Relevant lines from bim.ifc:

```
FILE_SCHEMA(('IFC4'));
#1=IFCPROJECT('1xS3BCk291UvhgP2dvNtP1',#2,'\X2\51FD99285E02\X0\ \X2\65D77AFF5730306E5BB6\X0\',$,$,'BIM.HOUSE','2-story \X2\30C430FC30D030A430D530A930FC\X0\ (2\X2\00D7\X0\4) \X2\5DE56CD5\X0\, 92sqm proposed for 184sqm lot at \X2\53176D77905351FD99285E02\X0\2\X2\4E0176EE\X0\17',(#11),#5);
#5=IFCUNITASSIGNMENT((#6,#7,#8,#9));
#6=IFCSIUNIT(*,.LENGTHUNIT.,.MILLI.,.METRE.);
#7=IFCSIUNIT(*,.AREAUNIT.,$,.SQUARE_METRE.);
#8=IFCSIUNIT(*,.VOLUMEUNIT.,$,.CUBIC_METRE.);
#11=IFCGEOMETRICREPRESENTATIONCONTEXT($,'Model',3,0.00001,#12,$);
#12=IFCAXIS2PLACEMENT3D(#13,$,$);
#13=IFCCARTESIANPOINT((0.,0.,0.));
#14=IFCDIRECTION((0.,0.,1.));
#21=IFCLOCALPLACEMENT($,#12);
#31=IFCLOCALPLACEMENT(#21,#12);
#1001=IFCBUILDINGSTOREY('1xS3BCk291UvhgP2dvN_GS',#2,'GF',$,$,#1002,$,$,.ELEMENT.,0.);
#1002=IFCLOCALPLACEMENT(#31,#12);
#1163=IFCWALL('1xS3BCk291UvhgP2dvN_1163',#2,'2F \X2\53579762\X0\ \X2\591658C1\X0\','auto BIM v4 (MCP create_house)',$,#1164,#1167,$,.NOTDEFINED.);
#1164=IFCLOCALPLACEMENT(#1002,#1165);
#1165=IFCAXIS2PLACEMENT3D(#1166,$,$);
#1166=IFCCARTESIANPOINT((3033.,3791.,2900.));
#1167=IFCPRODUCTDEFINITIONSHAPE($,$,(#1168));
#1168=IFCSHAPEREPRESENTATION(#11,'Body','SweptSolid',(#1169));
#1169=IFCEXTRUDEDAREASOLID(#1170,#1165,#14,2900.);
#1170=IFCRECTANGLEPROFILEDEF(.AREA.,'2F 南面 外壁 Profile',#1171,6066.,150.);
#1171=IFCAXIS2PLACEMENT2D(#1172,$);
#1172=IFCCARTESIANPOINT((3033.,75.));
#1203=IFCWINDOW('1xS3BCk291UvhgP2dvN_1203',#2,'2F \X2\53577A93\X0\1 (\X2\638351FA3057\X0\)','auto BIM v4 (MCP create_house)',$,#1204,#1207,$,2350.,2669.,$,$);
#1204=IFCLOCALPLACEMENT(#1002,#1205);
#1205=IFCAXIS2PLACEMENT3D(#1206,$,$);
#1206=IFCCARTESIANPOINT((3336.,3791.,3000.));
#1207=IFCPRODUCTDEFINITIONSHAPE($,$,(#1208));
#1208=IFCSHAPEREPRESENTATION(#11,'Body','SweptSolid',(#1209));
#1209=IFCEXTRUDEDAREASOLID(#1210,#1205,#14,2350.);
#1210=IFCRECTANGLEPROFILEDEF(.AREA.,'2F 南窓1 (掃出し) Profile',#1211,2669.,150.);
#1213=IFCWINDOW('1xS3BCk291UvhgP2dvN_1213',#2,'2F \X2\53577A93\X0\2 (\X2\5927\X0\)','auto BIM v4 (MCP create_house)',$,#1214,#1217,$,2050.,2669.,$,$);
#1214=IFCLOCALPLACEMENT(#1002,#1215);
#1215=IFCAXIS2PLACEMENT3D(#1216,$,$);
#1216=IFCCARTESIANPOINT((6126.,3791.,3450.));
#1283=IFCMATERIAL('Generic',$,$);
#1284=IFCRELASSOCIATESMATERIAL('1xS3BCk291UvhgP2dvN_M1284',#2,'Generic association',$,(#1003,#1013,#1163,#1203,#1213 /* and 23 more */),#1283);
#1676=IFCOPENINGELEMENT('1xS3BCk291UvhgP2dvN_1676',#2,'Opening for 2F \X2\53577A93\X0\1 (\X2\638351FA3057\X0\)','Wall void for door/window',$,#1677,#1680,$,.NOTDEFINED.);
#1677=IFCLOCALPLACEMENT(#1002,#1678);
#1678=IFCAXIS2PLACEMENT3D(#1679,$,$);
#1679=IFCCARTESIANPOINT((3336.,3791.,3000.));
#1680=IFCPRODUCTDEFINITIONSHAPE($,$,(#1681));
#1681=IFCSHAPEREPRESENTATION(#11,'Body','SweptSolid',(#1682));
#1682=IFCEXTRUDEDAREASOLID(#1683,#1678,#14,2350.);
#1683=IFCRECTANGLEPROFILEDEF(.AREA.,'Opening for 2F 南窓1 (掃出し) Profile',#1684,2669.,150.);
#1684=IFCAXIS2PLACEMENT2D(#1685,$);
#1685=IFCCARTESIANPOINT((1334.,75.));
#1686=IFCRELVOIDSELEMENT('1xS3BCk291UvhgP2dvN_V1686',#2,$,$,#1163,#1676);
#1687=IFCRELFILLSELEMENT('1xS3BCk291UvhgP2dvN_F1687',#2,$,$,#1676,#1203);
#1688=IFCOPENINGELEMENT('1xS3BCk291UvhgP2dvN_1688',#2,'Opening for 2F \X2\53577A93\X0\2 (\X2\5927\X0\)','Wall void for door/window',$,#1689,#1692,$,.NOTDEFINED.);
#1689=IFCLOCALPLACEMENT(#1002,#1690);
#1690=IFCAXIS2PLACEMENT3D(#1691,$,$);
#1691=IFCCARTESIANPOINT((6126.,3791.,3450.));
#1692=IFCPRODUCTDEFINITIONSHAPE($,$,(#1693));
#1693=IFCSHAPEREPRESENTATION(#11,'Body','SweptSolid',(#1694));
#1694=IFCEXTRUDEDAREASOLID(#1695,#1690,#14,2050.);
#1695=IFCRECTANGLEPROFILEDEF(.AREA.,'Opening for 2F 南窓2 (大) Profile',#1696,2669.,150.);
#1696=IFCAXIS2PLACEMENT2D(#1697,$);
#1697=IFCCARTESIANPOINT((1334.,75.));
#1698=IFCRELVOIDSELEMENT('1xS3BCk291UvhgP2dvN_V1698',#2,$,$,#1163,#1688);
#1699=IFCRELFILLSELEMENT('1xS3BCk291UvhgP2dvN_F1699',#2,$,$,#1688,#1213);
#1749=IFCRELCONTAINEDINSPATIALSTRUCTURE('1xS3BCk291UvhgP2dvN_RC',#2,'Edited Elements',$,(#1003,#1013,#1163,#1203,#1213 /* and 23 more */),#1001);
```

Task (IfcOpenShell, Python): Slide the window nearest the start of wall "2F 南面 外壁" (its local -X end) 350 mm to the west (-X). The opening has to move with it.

```python
import ifcopenshell
import ifcopenshell.api.geometry
import ifcopenshell.util.placement
import ifcopenshell.util.unit

model = ifcopenshell.open("bim.ifc")
unit_scale = ifcopenshell.util.unit.calculate_unit_scale(model)

window = model.by_guid("1xS3BCk291UvhgP2dvN_1203")
opening = window.FillsVoids[0].RelatingOpeningElement
wall = opening.VoidsElements[0].RelatingBuildingElement

wall_matrix = ifcopenshell.util.placement.get_local_placement(wall.ObjectPlacement)
shift = wall_matrix[:3, 0] * -0.35 / unit_scale
before = ifcopenshell.util.placement.get_local_placement(window.ObjectPlacement)[:3, 3].copy()

# The window is not placed relative to its opening, so move both.
for product in (opening, window):
    matrix = ifcopenshell.util.placement.get_local_placement(product.ObjectPlacement)
    matrix[:3, 3] += shift
    ifcopenshell.api.geometry.edit_object_placement(model, product=product, matrix=matrix, is_si=False)

after = ifcopenshell.util.placement.get_local_placement(window.ObjectPlacement)[:3, 3]
print("window moved by", (after - before).round(3) + 0.0)

model.write("bim-out.ifc")
```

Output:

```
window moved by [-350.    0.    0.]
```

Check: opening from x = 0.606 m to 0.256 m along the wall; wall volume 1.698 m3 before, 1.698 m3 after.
